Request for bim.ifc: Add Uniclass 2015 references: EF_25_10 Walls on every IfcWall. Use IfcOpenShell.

First a look at what the model holds.

```python
import ifcopenshell

model = ifcopenshell.open("bim.ifc")
print(model.schema)
print("classifications:", [c.Name for c in model.by_type("IfcClassification")])
for ifc_class in ("IfcDoor", "IfcRoof", "IfcStair", "IfcWall", "IfcWindow"):
    print(ifc_class, len(model.by_type(ifc_class)))
```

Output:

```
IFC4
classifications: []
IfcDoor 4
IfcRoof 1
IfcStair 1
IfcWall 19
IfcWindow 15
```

```python
import ifcopenshell
import ifcopenshell.api.classification

model = ifcopenshell.open("bim.ifc")

system = ifcopenshell.api.classification.add_classification(model, classification="Uniclass 2015")

codes = {
    "IfcWall": ("EF_25_10", "Walls"),
}
for ifc_class, (code, name) in codes.items():
    products = model.by_type(ifc_class)
    ifcopenshell.api.classification.add_reference(
        model, products=products, classification=system, identification=code, name=name
    )
    print(code, len(products))

model.write("bim_v2.ifc")
```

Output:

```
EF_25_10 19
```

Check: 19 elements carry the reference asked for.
